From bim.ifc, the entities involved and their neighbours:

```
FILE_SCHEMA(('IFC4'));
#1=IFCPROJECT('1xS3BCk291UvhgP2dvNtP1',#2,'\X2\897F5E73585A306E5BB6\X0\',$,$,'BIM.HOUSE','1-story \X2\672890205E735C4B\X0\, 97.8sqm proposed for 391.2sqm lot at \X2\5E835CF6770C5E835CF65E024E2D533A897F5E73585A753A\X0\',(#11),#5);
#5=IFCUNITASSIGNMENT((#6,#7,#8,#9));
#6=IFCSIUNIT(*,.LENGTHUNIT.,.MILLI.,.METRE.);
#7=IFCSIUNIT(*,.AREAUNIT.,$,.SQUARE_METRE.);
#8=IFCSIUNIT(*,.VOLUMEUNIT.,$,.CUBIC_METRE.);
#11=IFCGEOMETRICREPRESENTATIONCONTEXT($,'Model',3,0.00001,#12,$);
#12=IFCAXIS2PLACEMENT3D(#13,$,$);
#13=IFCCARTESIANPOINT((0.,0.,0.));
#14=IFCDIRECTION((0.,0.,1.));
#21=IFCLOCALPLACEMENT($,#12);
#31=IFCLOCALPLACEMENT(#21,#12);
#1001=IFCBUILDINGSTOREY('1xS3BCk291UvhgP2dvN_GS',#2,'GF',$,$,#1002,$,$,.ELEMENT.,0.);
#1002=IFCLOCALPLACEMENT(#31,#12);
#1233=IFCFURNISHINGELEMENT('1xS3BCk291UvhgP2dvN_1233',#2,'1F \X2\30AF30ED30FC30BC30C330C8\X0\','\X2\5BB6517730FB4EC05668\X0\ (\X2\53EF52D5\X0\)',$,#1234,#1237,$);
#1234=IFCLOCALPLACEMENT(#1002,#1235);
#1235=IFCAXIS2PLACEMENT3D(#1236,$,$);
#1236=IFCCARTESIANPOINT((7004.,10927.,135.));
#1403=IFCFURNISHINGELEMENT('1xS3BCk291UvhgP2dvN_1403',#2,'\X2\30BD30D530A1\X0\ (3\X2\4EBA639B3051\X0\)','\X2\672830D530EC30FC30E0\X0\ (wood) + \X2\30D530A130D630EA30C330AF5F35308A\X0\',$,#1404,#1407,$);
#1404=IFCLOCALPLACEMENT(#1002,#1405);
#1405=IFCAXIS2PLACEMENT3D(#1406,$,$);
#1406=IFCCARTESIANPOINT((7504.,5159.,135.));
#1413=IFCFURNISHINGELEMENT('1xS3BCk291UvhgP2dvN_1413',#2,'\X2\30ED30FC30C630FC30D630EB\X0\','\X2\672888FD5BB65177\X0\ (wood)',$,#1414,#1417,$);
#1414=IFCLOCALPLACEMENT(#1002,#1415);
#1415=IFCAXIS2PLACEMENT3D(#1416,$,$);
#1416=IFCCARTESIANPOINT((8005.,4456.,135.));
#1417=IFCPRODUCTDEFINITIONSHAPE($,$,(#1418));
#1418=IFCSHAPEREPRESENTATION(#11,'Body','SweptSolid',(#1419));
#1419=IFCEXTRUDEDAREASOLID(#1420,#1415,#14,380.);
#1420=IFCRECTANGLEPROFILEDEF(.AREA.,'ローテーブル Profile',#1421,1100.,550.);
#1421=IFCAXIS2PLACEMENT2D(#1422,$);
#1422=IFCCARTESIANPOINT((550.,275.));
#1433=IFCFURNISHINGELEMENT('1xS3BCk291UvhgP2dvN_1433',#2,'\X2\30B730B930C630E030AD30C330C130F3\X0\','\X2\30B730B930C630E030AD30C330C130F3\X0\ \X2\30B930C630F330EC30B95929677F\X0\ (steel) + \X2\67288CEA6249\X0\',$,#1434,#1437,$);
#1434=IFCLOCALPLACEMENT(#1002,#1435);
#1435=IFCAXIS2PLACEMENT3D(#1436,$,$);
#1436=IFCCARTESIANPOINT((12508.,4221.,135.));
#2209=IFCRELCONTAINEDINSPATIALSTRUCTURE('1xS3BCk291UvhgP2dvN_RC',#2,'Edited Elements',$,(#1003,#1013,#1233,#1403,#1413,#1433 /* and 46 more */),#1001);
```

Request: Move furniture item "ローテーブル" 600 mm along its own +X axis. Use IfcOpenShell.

```python
import ifcopenshell
import ifcopenshell.api.geometry
import ifcopenshell.util.placement
import ifcopenshell.util.unit

model = ifcopenshell.open("bim.ifc")
unit_scale = ifcopenshell.util.unit.calculate_unit_scale(model)

item = model.by_guid("1xS3BCk291UvhgP2dvN_1413")
matrix = ifcopenshell.util.placement.get_local_placement(item.ObjectPlacement)
matrix[:3, 3] += matrix[:3, 0] * 0.6 / unit_scale
ifcopenshell.api.geometry.edit_object_placement(model, product=item, matrix=matrix, is_si=False)

print(ifcopenshell.util.placement.get_local_placement(item.ObjectPlacement).round(3) + 0.0)

model.write("bim-out.ifc")
```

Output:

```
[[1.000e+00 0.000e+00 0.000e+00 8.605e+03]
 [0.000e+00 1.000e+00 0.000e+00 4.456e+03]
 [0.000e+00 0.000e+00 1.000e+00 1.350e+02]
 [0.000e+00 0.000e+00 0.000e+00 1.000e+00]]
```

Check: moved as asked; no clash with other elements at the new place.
